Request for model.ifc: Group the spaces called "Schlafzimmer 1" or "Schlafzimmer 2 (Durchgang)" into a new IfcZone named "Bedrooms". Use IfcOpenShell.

First a look at what the model holds.

```python
import ifcopenshell

model = ifcopenshell.open("model.ifc")
print(model.schema)
seen = {}
for space in model.by_type("IfcSpace"):
    seen[space.LongName] = seen.get(space.LongName, 0) + 1
for name, count in sorted(seen.items(), key=str):
    print(count, "x", name)
print("zones:", [z.Name for z in model.by_type("IfcZone")][:20])
```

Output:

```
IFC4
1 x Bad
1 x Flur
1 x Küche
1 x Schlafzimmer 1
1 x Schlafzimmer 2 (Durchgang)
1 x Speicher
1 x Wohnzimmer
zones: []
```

```python
import ifcopenshell
import ifcopenshell.api.group
import ifcopenshell.api.root

model = ifcopenshell.open("model.ifc")

names = {"Schlafzimmer 1", "Schlafzimmer 2 (Durchgang)"}
spaces = [s for s in model.by_type("IfcSpace") if s.LongName in names]

zone = ifcopenshell.api.root.create_entity(model, ifc_class="IfcZone", name="Bedrooms")
ifcopenshell.api.group.assign_group(model, products=spaces, group=zone)
print(len(spaces), "spaces in", zone.Name)

model.write("model_rev.ifc")
```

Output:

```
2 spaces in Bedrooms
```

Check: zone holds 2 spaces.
